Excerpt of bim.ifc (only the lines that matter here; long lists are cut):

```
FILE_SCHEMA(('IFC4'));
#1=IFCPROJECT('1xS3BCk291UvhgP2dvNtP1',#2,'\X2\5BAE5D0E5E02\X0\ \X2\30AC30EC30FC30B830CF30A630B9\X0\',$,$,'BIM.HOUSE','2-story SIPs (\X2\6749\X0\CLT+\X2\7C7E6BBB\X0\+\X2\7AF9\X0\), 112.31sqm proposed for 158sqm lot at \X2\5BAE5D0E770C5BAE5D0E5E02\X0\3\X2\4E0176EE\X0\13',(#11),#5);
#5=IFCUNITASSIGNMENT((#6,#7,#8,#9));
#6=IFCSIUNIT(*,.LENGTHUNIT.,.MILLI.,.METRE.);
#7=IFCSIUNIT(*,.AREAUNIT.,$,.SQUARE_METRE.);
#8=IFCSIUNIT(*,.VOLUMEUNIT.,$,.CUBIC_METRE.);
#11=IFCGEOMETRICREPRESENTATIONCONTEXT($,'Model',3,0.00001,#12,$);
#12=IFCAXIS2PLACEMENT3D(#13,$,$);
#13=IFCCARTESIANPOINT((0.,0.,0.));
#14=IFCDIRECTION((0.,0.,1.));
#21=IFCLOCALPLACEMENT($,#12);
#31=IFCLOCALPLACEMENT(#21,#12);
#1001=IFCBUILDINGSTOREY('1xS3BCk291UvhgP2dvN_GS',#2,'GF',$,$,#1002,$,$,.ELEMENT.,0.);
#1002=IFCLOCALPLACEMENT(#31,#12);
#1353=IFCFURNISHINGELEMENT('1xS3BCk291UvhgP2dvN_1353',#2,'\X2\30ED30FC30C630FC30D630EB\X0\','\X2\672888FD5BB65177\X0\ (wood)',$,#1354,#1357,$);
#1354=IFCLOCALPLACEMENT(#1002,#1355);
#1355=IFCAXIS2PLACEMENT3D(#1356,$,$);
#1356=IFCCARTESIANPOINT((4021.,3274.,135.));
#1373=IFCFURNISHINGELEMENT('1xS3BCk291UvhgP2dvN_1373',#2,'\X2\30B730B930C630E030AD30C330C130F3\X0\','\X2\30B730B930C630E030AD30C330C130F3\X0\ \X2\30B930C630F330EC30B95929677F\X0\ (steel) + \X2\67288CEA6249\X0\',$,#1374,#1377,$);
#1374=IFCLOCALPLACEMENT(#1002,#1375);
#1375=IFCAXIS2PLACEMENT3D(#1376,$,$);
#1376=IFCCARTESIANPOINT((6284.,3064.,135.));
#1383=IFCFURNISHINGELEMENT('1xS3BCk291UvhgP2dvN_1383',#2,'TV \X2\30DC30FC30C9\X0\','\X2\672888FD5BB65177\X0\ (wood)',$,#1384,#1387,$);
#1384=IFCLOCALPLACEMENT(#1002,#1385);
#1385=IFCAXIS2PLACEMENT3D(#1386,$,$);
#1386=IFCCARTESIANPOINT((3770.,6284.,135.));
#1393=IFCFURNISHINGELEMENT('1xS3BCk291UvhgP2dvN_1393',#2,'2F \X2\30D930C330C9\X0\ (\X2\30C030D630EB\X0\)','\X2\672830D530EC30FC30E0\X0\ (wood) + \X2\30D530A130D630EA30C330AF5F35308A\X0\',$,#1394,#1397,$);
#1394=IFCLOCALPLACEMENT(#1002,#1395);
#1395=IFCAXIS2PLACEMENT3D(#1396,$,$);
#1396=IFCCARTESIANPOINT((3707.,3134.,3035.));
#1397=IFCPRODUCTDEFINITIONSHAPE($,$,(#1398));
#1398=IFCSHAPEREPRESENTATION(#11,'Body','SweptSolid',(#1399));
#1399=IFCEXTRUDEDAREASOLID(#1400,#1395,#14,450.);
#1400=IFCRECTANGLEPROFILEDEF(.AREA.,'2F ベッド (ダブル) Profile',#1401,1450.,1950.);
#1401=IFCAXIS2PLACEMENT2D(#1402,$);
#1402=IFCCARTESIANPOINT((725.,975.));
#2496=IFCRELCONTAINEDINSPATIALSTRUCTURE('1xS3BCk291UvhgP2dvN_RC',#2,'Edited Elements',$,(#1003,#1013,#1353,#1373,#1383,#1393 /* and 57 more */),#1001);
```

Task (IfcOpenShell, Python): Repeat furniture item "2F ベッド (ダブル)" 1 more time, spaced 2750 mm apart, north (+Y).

```python
import numpy as np
import ifcopenshell
import ifcopenshell.api.geometry
import ifcopenshell.api.root
import ifcopenshell.util.element
import ifcopenshell.util.placement
import ifcopenshell.util.unit

model = ifcopenshell.open("bim.ifc")
unit_scale = ifcopenshell.util.unit.calculate_unit_scale(model)


def reuse_history(source, copy):
    """copy_class also copies each property set's owner history, people and application; keep the originals."""
    for rel in copy.IsDefinedBy:
        if rel.is_a("IfcRelDefinesByProperties") and (history := rel.RelatingPropertyDefinition.OwnerHistory):
            rel.RelatingPropertyDefinition.OwnerHistory = source.OwnerHistory
            ifcopenshell.util.element.remove_deep2(model, history)


source = model.by_guid("1xS3BCk291UvhgP2dvN_1393")
base = ifcopenshell.util.placement.get_local_placement(source.ObjectPlacement)
step = np.array([0.0, 1.0, 0.0]) * 2.75 / unit_scale

for i in range(1, 2):
    copy = ifcopenshell.api.root.copy_class(model, product=source)
    copy.Representation = ifcopenshell.util.element.copy_deep(
        model, source.Representation, exclude=["IfcGeometricRepresentationContext", "IfcRepresentationMap"]
    )
    reuse_history(source, copy)
    matrix = base.copy()
    matrix[:3, 3] += i * step
    print("added at", matrix[:3, 3].round(3) + 0.0)
    ifcopenshell.api.geometry.edit_object_placement(model, product=copy, matrix=matrix, is_si=False)

model.write("bim-out.ifc")
```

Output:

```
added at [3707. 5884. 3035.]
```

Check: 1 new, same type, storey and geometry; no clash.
